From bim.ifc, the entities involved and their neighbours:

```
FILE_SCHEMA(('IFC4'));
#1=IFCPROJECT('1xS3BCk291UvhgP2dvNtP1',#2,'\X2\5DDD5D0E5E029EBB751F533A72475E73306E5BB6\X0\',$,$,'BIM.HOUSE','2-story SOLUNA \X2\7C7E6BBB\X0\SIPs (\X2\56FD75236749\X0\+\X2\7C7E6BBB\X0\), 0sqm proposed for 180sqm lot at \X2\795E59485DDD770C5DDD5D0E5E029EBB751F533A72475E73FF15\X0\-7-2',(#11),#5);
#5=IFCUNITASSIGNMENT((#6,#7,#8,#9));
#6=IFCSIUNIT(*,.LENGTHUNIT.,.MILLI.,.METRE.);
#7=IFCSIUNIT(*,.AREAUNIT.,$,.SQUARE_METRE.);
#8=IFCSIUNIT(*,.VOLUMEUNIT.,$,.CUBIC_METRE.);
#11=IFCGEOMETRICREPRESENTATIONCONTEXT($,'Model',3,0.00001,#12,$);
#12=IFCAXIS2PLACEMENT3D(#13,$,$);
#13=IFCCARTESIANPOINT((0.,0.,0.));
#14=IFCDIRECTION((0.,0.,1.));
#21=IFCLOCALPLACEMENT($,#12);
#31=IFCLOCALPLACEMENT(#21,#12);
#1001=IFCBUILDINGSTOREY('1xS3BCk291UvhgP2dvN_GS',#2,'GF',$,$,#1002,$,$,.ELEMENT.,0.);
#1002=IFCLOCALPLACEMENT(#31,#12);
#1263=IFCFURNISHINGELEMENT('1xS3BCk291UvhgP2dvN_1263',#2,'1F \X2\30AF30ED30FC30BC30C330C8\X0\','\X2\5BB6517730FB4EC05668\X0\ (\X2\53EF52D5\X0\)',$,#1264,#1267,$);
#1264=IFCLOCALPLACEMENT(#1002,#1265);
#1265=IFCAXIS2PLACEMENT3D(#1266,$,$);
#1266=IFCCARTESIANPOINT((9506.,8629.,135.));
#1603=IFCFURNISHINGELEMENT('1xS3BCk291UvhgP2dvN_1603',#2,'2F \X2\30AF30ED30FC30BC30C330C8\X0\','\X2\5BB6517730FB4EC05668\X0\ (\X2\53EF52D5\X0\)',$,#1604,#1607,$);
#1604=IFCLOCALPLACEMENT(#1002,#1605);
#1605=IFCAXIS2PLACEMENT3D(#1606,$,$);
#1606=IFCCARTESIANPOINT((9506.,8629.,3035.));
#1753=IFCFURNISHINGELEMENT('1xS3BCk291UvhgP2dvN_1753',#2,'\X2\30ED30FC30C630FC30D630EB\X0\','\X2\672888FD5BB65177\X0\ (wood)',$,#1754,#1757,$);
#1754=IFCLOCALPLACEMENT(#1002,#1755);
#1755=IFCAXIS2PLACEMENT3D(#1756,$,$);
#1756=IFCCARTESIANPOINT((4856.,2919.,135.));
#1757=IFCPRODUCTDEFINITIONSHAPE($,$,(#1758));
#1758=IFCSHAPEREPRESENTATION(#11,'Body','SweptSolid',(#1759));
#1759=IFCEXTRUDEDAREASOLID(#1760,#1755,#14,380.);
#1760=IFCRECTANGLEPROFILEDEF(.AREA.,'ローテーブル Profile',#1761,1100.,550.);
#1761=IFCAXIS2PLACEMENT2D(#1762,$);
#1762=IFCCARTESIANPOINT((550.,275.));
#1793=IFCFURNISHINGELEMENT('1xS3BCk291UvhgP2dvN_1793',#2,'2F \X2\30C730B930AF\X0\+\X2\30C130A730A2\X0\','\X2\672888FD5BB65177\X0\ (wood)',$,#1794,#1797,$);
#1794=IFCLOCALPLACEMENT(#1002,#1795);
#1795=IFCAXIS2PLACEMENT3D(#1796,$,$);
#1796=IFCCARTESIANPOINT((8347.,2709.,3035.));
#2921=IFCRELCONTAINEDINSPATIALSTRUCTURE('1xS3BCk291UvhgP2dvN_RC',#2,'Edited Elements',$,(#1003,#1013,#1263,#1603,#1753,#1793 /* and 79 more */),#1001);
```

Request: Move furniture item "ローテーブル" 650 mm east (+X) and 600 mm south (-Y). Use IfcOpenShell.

```python
import ifcopenshell
import ifcopenshell.api.geometry
import ifcopenshell.util.placement
import ifcopenshell.util.unit

model = ifcopenshell.open("bim.ifc")
unit_scale = ifcopenshell.util.unit.calculate_unit_scale(model)

item = model.by_id(1753)
matrix = ifcopenshell.util.placement.get_local_placement(item.ObjectPlacement)
matrix[0, 3] += 0.65 / unit_scale
matrix[1, 3] -= 0.6 / unit_scale
ifcopenshell.api.geometry.edit_object_placement(model, product=item, matrix=matrix, is_si=False)

print(ifcopenshell.util.placement.get_local_placement(item.ObjectPlacement).round(3) + 0.0)

model.write("bim_v2.ifc")
```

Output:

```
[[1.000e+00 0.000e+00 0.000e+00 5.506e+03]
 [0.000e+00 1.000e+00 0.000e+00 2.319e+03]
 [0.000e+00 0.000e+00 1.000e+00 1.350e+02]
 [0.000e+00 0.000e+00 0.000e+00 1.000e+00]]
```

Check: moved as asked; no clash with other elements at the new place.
